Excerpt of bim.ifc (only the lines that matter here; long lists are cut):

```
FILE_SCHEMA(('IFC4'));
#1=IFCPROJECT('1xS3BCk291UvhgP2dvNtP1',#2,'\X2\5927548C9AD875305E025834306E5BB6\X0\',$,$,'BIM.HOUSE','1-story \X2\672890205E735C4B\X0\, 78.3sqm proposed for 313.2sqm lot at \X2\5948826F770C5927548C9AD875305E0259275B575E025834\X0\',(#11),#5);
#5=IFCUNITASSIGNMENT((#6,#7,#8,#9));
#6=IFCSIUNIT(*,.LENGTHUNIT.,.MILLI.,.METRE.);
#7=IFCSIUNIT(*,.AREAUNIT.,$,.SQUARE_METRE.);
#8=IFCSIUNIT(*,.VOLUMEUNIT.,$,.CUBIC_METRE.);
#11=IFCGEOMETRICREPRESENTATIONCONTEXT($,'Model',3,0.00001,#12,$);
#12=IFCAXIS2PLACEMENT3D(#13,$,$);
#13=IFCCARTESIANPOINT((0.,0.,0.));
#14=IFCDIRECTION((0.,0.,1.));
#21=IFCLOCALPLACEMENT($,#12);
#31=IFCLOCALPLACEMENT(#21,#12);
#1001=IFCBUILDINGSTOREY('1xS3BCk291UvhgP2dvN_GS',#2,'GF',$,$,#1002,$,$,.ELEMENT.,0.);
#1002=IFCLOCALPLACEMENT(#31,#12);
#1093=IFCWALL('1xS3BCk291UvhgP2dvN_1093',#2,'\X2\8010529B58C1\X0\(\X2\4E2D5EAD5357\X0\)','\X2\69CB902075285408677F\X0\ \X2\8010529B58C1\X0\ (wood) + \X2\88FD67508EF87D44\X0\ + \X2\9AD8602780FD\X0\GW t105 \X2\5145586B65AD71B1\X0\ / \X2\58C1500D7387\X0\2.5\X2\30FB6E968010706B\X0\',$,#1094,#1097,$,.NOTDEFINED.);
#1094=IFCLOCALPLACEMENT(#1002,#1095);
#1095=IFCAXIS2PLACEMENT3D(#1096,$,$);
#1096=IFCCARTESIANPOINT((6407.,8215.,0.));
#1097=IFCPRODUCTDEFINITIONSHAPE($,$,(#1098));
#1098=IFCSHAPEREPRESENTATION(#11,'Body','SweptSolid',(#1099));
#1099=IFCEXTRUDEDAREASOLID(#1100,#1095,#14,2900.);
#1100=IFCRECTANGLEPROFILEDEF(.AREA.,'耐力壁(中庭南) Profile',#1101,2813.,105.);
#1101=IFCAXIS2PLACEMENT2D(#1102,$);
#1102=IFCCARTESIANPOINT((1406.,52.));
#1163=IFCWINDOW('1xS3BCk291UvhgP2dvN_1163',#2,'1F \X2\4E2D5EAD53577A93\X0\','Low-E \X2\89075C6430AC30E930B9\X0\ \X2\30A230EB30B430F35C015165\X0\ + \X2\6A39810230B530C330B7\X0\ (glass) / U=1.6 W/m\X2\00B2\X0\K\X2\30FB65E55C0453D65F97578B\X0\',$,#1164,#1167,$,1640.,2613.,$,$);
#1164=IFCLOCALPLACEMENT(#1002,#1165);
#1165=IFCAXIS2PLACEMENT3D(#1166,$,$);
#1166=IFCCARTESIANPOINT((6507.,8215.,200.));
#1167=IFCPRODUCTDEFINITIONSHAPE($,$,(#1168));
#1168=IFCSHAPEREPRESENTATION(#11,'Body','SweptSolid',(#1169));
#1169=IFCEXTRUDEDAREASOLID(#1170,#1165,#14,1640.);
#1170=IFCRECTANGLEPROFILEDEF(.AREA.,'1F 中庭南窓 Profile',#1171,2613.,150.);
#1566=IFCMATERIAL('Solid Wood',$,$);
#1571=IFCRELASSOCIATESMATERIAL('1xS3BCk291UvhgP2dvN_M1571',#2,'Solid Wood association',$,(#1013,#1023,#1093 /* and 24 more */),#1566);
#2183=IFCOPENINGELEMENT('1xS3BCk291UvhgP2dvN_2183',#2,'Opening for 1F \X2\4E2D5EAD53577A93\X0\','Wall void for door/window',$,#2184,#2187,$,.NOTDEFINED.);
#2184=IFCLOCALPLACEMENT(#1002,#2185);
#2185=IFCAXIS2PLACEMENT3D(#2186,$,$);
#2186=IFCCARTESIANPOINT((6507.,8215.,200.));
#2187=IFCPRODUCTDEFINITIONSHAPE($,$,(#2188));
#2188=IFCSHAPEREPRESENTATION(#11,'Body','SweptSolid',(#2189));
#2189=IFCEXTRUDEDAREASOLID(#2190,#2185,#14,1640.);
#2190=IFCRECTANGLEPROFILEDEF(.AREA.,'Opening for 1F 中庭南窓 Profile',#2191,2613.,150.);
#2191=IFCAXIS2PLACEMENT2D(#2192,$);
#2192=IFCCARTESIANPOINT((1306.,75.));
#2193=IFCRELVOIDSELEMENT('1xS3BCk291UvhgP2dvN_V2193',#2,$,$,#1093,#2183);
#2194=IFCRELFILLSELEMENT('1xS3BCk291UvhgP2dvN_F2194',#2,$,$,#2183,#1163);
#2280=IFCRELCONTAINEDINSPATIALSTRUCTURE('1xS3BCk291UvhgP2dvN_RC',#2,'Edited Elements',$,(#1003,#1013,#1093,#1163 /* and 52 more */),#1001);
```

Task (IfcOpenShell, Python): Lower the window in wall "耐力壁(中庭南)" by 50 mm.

```python
import numpy as np
import ifcopenshell
import ifcopenshell.api.geometry
import ifcopenshell.util.placement
import ifcopenshell.util.unit

model = ifcopenshell.open("bim.ifc")
unit_scale = ifcopenshell.util.unit.calculate_unit_scale(model)

window = model.by_guid("1xS3BCk291UvhgP2dvN_1163")
opening = window.FillsVoids[0].RelatingOpeningElement
dz = -0.05 / unit_scale

shift = np.array([0.0, 0.0, dz])
# The window is not placed relative to its opening, so move both.
for product in (opening, window):
    matrix = ifcopenshell.util.placement.get_local_placement(product.ObjectPlacement)
    matrix[:3, 3] += shift
    ifcopenshell.api.geometry.edit_object_placement(model, product=product, matrix=matrix, is_si=False)

print(f"moved by {dz * unit_scale:+.3f} m")

model.write("bim_v2.ifc")
```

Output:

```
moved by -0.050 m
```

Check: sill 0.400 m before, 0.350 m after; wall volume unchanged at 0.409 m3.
